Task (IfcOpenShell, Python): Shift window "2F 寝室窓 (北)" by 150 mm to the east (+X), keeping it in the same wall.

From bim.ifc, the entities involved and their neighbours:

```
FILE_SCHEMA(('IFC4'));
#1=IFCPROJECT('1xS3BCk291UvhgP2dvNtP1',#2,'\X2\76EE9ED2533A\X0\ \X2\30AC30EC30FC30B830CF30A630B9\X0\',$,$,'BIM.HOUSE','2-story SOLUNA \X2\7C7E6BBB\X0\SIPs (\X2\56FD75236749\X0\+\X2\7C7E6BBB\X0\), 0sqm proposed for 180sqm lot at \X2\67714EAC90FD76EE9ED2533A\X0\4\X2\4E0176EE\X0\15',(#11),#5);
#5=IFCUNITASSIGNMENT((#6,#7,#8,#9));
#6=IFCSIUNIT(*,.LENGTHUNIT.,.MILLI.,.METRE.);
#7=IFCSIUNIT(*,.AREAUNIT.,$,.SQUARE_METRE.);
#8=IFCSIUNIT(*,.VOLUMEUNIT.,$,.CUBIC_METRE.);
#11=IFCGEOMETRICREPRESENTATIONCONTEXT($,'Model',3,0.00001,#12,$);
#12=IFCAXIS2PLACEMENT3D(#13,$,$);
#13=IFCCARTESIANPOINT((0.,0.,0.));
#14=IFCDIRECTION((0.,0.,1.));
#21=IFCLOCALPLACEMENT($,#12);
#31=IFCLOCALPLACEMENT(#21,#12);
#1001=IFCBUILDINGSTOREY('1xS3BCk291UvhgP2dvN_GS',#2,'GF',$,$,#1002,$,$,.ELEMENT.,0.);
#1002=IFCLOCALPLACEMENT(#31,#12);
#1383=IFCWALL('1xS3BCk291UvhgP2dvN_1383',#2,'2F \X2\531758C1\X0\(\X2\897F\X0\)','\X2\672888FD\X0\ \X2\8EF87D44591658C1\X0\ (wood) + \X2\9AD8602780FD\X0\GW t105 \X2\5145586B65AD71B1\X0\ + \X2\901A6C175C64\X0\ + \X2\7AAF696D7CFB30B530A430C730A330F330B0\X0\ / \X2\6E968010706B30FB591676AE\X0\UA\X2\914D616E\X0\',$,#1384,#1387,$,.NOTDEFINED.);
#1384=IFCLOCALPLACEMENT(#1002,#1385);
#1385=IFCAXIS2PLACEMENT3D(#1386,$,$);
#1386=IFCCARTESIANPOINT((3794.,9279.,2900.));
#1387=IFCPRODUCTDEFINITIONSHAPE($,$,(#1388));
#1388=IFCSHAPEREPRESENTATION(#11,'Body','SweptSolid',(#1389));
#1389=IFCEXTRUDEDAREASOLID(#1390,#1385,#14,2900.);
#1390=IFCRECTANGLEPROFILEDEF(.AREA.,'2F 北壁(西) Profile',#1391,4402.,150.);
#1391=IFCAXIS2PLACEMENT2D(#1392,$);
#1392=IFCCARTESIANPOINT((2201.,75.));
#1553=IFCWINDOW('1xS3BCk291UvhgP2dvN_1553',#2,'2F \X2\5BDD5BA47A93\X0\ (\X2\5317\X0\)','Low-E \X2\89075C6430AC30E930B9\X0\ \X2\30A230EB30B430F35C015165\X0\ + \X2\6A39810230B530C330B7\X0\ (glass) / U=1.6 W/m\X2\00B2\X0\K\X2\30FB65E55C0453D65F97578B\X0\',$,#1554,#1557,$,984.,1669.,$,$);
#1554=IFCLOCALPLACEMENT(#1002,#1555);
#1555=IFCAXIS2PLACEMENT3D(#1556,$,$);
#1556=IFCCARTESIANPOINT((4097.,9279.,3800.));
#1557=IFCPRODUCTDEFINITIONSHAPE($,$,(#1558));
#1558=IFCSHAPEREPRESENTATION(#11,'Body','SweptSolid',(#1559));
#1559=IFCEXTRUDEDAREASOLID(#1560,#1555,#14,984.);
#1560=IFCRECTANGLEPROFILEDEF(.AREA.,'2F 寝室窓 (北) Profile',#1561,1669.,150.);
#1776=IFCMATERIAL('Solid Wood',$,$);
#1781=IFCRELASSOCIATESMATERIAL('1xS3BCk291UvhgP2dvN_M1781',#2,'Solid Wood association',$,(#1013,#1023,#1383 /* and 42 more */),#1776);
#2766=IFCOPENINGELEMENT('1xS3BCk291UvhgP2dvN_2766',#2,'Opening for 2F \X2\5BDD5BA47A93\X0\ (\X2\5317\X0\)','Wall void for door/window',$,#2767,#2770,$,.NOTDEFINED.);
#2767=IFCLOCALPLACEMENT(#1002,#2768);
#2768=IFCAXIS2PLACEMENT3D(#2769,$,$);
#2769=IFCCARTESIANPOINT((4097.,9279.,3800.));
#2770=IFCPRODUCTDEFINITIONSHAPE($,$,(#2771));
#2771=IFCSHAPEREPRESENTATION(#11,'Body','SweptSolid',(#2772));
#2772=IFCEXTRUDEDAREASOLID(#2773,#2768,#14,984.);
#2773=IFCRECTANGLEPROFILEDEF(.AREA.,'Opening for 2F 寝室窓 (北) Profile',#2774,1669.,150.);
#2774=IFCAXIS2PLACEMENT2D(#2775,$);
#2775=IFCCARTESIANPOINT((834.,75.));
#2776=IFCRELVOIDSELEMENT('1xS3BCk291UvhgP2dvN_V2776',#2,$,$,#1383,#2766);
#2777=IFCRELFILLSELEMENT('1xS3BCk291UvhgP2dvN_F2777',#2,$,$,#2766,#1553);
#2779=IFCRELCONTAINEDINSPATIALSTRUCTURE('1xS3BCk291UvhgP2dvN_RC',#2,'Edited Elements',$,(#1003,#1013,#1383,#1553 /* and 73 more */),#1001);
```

```python
import ifcopenshell
import ifcopenshell.api.geometry
import ifcopenshell.util.placement
import ifcopenshell.util.unit

model = ifcopenshell.open("bim.ifc")
unit_scale = ifcopenshell.util.unit.calculate_unit_scale(model)

window = model.by_id(1553)
opening = window.FillsVoids[0].RelatingOpeningElement
wall = opening.VoidsElements[0].RelatingBuildingElement

wall_matrix = ifcopenshell.util.placement.get_local_placement(wall.ObjectPlacement)
shift = wall_matrix[:3, 0] * 0.15 / unit_scale
before = ifcopenshell.util.placement.get_local_placement(window.ObjectPlacement)[:3, 3].copy()

# The window is not placed relative to its opening, so move both.
for product in (opening, window):
    matrix = ifcopenshell.util.placement.get_local_placement(product.ObjectPlacement)
    matrix[:3, 3] += shift
    ifcopenshell.api.geometry.edit_object_placement(model, product=product, matrix=matrix, is_si=False)

after = ifcopenshell.util.placement.get_local_placement(window.ObjectPlacement)[:3, 3]
print("window moved by", (after - before).round(3) + 0.0)

model.write("bim_rev.ifc")
```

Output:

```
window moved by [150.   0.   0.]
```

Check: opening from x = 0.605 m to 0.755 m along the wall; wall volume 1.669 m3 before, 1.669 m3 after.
